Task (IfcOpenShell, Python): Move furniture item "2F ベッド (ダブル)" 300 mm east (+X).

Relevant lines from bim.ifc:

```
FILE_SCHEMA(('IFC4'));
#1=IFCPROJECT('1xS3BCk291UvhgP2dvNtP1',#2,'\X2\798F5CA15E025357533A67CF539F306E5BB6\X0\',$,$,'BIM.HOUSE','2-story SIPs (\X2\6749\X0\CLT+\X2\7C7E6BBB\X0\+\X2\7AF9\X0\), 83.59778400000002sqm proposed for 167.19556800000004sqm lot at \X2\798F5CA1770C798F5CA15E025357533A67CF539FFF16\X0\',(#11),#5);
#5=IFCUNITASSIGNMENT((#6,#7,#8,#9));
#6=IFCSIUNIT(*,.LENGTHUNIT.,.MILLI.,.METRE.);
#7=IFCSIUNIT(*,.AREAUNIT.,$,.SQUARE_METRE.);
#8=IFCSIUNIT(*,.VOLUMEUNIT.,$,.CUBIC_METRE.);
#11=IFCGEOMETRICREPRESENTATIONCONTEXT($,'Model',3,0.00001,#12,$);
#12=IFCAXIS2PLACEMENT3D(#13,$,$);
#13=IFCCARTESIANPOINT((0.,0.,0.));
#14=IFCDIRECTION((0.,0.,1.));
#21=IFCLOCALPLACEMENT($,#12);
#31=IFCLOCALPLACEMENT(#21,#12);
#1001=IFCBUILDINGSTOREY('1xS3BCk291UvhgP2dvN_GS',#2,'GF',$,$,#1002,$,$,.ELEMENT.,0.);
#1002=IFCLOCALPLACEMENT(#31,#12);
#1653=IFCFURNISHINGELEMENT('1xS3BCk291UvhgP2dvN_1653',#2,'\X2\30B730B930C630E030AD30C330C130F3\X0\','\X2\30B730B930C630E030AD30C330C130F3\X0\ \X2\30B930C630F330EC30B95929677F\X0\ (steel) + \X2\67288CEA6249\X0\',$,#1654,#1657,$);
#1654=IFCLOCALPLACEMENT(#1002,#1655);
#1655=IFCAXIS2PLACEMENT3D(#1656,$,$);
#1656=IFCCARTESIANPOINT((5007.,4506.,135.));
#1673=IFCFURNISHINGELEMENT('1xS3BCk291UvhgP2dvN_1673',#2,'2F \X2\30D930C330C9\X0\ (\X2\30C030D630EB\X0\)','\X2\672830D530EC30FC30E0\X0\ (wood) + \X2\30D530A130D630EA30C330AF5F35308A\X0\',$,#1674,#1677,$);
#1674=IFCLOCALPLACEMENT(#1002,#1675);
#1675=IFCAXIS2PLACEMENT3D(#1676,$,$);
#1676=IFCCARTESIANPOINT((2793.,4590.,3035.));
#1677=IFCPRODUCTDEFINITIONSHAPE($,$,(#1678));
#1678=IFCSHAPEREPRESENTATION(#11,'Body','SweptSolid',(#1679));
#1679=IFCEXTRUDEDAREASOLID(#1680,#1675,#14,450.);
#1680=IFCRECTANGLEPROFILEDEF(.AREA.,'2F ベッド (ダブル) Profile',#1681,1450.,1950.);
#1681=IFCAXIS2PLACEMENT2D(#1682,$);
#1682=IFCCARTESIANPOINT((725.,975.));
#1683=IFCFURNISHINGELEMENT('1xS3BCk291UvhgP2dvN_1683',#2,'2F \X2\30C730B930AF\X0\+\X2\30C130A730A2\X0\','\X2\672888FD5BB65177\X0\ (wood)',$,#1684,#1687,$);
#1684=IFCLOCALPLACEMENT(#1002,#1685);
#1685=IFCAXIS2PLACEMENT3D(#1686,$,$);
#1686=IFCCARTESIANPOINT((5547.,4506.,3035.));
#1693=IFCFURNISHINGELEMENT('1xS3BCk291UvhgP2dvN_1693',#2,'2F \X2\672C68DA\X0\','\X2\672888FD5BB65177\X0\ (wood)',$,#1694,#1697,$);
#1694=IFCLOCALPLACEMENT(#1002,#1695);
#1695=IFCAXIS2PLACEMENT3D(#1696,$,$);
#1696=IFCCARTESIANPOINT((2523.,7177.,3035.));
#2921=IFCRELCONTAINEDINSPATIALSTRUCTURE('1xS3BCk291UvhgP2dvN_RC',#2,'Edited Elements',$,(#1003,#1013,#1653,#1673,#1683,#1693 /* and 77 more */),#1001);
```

```python
import ifcopenshell
import ifcopenshell.api.geometry
import ifcopenshell.util.placement
import ifcopenshell.util.unit

model = ifcopenshell.open("bim.ifc")
unit_scale = ifcopenshell.util.unit.calculate_unit_scale(model)

item = model.by_guid("1xS3BCk291UvhgP2dvN_1673")
matrix = ifcopenshell.util.placement.get_local_placement(item.ObjectPlacement)
matrix[0, 3] += 0.3 / unit_scale
ifcopenshell.api.geometry.edit_object_placement(model, product=item, matrix=matrix, is_si=False)

print(ifcopenshell.util.placement.get_local_placement(item.ObjectPlacement).round(3) + 0.0)

model.write("bim_edited.ifc")
```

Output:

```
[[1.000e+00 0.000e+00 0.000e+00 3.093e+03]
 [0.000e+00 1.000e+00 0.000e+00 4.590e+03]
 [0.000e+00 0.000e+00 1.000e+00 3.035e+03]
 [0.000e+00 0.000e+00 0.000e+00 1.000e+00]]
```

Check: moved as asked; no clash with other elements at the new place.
